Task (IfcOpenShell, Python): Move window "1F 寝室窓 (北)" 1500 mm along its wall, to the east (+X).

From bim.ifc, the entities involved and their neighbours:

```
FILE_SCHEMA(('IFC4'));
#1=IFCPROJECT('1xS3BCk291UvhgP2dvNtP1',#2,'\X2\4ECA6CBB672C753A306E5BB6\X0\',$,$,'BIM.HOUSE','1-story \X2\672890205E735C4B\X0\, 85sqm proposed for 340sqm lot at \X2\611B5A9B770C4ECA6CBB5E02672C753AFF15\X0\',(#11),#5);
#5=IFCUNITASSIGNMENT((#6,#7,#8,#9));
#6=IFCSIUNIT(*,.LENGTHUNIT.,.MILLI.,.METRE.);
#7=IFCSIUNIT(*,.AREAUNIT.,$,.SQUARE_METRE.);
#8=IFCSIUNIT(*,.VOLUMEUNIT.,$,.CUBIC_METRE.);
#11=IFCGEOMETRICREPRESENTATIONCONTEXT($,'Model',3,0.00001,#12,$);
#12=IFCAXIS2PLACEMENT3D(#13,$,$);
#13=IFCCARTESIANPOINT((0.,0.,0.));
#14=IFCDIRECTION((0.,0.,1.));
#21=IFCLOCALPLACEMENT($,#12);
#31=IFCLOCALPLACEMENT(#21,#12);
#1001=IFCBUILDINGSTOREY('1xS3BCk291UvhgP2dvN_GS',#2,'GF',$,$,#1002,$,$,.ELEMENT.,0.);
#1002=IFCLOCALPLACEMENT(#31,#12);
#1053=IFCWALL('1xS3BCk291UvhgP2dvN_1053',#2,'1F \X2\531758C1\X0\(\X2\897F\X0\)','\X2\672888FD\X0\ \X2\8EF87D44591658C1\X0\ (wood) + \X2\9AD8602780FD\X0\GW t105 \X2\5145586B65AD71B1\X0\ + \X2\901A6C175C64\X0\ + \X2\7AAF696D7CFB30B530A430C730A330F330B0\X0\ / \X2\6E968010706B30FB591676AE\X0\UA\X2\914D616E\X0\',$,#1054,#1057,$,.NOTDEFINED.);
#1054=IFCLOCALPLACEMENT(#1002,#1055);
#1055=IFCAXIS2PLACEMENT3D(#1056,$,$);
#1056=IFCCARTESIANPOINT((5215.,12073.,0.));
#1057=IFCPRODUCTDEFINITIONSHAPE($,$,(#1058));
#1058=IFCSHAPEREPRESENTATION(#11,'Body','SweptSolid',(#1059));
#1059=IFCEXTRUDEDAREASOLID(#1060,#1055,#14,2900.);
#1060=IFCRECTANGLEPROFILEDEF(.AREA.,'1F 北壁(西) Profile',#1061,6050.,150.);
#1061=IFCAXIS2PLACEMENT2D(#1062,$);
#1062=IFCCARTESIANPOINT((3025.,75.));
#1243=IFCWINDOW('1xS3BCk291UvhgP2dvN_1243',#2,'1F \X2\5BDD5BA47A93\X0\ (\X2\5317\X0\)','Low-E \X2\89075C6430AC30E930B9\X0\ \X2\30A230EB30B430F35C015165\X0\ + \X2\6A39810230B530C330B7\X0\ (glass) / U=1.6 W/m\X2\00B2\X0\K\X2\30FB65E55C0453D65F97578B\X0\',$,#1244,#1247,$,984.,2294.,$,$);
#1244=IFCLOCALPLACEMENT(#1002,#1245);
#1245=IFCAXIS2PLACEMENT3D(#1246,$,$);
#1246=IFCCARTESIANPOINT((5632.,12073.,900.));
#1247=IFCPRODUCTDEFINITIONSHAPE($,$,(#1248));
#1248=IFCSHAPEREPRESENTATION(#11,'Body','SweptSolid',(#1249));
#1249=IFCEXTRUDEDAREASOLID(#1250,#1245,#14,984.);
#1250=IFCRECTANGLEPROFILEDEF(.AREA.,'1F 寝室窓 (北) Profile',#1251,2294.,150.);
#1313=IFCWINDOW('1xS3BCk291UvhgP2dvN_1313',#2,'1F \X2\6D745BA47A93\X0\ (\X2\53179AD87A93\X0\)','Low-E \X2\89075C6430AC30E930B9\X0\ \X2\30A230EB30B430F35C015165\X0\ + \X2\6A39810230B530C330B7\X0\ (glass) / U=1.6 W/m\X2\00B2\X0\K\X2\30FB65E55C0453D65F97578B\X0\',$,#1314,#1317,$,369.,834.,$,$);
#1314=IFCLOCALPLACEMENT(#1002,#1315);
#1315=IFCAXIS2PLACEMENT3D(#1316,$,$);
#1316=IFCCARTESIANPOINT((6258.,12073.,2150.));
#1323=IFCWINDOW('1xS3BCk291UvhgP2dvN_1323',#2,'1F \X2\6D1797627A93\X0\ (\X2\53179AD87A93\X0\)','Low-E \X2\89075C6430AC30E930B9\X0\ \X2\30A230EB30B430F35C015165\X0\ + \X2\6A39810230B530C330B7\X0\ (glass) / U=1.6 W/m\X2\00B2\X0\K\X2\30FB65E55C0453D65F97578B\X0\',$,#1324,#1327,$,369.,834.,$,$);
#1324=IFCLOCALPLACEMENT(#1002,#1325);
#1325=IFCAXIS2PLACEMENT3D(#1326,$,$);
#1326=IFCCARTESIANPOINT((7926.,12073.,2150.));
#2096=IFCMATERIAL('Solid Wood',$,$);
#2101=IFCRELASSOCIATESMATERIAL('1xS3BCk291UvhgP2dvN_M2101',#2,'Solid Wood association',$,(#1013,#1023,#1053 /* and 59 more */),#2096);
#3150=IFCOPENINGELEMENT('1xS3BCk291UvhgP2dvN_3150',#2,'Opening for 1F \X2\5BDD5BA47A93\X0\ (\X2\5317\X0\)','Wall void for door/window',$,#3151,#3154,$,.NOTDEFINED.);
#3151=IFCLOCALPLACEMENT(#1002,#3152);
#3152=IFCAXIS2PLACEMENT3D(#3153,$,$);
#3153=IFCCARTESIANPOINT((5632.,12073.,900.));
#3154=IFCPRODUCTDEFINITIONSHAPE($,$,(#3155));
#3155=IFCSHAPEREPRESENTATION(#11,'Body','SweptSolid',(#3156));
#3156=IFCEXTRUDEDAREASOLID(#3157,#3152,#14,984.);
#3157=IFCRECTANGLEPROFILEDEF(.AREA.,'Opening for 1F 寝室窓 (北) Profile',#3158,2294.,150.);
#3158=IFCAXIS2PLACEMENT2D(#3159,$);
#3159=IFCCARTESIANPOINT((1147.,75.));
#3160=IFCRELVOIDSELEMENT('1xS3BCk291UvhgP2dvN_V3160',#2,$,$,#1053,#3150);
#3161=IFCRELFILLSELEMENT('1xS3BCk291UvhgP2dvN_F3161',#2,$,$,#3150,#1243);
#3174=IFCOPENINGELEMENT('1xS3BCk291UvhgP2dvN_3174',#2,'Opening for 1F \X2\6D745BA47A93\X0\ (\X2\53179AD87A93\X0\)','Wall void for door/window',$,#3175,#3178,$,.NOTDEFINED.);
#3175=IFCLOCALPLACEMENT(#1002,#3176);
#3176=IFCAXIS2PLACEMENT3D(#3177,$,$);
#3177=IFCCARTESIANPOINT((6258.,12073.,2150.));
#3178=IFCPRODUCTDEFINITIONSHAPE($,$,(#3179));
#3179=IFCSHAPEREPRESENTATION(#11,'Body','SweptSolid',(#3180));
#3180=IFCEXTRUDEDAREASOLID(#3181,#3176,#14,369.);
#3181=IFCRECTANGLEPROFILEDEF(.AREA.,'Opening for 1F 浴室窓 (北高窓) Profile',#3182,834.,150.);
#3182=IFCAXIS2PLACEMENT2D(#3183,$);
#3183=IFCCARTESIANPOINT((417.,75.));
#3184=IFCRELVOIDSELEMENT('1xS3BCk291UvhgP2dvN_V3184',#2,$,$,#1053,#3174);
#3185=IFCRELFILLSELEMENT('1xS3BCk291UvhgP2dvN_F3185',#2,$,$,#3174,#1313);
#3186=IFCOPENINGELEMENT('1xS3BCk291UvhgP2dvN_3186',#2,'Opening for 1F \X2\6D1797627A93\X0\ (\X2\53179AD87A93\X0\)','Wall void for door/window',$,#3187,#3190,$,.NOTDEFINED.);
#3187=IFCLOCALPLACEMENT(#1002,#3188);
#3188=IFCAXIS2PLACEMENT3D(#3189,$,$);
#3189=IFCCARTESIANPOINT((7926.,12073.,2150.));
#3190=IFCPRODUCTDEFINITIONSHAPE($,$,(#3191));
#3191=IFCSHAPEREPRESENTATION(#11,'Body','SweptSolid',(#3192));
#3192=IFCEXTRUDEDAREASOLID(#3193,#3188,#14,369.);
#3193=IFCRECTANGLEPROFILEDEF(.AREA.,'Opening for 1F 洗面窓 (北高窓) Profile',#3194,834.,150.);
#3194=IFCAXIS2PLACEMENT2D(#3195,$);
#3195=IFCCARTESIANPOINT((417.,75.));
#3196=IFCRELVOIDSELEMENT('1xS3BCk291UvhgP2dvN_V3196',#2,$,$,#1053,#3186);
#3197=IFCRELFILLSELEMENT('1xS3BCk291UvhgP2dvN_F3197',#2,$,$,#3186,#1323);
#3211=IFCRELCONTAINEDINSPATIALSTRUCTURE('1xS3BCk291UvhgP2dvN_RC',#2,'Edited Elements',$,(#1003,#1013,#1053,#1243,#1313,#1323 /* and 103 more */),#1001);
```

```python
import ifcopenshell
import ifcopenshell.api.geometry
import ifcopenshell.util.placement

model = ifcopenshell.open("bim.ifc")

window = model.by_guid("1xS3BCk291UvhgP2dvN_1243")
opening = window.FillsVoids[0].RelatingOpeningElement
wall = opening.VoidsElements[0].RelatingBuildingElement

wall_matrix = ifcopenshell.util.placement.get_local_placement(wall.ObjectPlacement)
shift = wall_matrix[:3, 0] * 1500.0
before = ifcopenshell.util.placement.get_local_placement(window.ObjectPlacement)[:3, 3].copy()

# The window is not placed relative to its opening, so move both.
for product in (opening, window):
    matrix = ifcopenshell.util.placement.get_local_placement(product.ObjectPlacement)
    matrix[:3, 3] += shift
    ifcopenshell.api.geometry.edit_object_placement(model, product=product, matrix=matrix, is_si=False)

after = ifcopenshell.util.placement.get_local_placement(window.ObjectPlacement)[:3, 3]
print("window moved by", (after - before).round(3) + 0.0)

model.write("bim_rev.ifc")
```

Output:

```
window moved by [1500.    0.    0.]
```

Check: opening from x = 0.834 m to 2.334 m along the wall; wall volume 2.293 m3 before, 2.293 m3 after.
